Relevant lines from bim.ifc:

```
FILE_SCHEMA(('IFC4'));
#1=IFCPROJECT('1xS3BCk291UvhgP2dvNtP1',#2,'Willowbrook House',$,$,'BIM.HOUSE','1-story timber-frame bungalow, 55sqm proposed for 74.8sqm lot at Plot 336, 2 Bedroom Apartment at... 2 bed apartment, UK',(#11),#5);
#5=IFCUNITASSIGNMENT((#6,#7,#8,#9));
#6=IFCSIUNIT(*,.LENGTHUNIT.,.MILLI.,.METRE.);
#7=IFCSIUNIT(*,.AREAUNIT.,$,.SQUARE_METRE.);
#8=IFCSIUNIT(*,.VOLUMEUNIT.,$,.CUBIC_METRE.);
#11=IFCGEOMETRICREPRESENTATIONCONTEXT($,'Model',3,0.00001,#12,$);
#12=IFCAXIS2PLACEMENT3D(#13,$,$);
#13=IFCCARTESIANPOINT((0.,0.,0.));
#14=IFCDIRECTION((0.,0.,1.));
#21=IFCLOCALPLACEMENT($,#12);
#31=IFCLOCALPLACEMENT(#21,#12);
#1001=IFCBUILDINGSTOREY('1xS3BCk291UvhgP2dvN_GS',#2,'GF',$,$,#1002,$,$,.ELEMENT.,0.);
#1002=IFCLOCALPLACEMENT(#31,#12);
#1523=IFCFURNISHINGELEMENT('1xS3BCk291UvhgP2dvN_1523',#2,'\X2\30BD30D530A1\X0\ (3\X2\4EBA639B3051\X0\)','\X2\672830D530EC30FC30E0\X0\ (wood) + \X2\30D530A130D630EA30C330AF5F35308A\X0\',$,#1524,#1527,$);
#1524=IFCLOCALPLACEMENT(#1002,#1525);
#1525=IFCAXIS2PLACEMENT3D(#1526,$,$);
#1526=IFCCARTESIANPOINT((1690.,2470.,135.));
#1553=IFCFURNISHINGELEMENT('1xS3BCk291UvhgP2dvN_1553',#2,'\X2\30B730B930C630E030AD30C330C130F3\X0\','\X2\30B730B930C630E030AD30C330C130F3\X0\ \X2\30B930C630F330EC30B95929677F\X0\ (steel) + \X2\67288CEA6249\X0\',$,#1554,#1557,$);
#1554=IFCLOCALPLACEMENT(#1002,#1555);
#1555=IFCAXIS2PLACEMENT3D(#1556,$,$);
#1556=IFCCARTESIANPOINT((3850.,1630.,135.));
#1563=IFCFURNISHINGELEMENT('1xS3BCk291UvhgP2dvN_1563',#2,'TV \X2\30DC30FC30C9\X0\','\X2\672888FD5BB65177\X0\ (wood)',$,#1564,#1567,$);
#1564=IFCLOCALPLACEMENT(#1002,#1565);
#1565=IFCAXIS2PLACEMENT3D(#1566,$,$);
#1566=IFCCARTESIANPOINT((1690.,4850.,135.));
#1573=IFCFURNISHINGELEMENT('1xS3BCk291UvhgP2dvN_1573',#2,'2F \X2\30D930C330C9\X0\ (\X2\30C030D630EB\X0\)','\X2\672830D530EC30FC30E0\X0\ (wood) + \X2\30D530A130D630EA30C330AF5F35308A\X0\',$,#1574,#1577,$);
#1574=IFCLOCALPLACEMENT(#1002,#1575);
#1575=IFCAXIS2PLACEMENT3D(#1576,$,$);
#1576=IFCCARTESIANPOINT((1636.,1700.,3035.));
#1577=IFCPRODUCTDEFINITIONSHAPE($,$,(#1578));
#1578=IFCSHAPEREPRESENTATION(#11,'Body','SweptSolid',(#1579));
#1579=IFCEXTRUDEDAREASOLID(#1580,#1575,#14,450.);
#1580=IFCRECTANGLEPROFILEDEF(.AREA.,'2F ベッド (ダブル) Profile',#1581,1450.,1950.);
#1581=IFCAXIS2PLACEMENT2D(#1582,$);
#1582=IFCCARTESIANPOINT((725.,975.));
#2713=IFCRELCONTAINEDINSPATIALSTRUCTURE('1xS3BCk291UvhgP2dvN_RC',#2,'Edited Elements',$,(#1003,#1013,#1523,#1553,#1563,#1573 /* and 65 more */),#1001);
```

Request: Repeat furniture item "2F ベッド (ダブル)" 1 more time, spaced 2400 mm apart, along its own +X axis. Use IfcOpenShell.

```python
import ifcopenshell
import ifcopenshell.api.geometry
import ifcopenshell.api.root
import ifcopenshell.util.element
import ifcopenshell.util.placement

model = ifcopenshell.open("bim.ifc")


def reuse_history(source, copy):
    """copy_class also copies each property set's owner history, people and application; keep the originals."""
    for rel in copy.IsDefinedBy:
        if rel.is_a("IfcRelDefinesByProperties") and (history := rel.RelatingPropertyDefinition.OwnerHistory):
            rel.RelatingPropertyDefinition.OwnerHistory = source.OwnerHistory
            ifcopenshell.util.element.remove_deep2(model, history)


source = model.by_id(1573)
base = ifcopenshell.util.placement.get_local_placement(source.ObjectPlacement)
step = base[:3, 0] * 2400.0

for i in range(1, 2):
    copy = ifcopenshell.api.root.copy_class(model, product=source)
    copy.Representation = ifcopenshell.util.element.copy_deep(
        model, source.Representation, exclude=["IfcGeometricRepresentationContext", "IfcRepresentationMap"]
    )
    reuse_history(source, copy)
    matrix = base.copy()
    matrix[:3, 3] += i * step
    print("added at", matrix[:3, 3].round(3) + 0.0)
    ifcopenshell.api.geometry.edit_object_placement(model, product=copy, matrix=matrix, is_si=False)

model.write("bim_updated.ifc")
```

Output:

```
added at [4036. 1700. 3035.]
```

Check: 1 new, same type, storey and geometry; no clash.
